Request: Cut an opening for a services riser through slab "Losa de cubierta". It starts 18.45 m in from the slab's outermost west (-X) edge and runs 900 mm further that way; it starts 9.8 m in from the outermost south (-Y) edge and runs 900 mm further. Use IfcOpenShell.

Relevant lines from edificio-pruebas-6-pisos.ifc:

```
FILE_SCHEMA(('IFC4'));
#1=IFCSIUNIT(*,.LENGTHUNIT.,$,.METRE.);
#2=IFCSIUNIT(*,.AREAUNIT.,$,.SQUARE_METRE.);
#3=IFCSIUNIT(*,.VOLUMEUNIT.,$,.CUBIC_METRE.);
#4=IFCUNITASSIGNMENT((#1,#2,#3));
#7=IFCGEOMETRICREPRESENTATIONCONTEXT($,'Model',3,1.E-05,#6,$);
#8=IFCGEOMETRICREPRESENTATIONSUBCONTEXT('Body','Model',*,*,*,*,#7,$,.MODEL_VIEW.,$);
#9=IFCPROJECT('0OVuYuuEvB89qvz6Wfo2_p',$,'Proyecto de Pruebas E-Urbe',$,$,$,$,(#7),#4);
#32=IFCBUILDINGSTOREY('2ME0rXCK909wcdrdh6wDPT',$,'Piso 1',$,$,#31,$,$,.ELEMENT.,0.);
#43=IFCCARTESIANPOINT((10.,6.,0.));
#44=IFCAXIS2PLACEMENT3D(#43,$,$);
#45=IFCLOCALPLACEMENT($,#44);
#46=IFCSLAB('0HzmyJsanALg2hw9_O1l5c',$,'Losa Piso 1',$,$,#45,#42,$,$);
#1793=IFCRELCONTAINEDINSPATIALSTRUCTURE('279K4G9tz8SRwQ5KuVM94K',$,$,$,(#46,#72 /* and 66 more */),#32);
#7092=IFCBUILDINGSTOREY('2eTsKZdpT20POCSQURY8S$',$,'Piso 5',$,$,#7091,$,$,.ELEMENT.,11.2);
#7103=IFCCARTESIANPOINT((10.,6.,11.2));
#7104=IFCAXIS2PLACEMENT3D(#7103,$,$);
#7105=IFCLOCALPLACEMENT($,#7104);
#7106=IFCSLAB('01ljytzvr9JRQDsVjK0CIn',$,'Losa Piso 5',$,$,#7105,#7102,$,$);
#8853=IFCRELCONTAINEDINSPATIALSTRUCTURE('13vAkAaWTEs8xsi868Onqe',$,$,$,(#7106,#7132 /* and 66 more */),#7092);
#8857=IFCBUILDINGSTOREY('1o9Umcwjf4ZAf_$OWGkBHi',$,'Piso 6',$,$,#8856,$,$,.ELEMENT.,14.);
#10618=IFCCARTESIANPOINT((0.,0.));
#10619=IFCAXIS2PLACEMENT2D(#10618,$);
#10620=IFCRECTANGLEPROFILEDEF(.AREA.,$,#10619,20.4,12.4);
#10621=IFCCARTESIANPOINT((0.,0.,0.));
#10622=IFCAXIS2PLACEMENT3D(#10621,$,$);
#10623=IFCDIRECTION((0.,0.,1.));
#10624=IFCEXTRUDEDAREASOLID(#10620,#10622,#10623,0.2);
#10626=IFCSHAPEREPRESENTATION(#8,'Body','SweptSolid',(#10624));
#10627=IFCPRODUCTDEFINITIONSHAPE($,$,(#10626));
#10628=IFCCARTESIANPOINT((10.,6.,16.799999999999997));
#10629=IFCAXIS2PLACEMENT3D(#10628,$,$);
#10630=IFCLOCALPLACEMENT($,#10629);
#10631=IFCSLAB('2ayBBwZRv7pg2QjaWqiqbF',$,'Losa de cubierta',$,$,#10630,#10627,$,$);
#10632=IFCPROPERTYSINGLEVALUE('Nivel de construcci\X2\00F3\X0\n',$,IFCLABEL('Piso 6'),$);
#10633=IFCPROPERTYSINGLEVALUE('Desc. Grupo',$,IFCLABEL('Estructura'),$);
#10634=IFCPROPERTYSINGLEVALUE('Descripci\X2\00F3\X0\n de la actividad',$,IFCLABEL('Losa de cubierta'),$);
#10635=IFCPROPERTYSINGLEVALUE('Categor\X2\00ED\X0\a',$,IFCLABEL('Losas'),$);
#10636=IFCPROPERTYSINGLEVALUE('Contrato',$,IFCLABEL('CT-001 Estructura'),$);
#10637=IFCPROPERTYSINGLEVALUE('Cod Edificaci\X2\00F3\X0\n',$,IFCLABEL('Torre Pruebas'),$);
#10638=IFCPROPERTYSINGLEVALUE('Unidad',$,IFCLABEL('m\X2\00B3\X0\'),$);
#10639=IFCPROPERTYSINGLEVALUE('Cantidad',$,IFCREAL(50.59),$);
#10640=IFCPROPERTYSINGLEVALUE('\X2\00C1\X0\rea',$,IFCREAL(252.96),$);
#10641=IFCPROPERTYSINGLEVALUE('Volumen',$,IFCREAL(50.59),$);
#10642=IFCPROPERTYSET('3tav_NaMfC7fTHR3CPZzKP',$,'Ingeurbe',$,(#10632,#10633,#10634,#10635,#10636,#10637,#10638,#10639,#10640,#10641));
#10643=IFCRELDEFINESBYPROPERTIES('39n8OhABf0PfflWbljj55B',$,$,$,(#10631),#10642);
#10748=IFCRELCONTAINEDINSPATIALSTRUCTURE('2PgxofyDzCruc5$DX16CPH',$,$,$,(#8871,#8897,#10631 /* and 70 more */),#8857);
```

```python
import numpy as np
import ifcopenshell
import ifcopenshell.api.feature
import ifcopenshell.api.geometry
import ifcopenshell.api.pset
import ifcopenshell.api.root
import ifcopenshell.geom
import ifcopenshell.util.element
import ifcopenshell.util.placement
import ifcopenshell.util.representation
import ifcopenshell.util.shape
import ifcopenshell.util.unit

model = ifcopenshell.open("edificio-pruebas-6-pisos.ifc")
unit_scale = ifcopenshell.util.unit.calculate_unit_scale(model)
area_scale = ifcopenshell.util.unit.calculate_unit_scale(model, "AREAUNIT")
volume_scale = ifcopenshell.util.unit.calculate_unit_scale(model, "VOLUMEUNIT")
settings = ifcopenshell.geom.settings()


def volume(element):
    """Net volume in cubic metres, openings subtracted."""
    shape = ifcopenshell.geom.create_shape(settings, element)
    return ifcopenshell.util.shape.get_volume(shape.geometry)


slab = model.by_guid("2ayBBwZRv7pg2QjaWqiqbF")
before = volume(slab)

# Extent in the slab's own axes, in metres. The edges named are its -X and -Y sides.
slab_shape = ifcopenshell.geom.create_shape(settings, slab)
vertices = ifcopenshell.util.shape.get_vertices(slab_shape.geometry)
x_min, y_min, bottom = vertices.min(axis=0)
top = vertices[:, 2].max()

opening = ifcopenshell.api.root.create_entity(model, ifc_class="IfcOpeningElement", name="Services riser opening", predefined_type="OPENING")
context = ifcopenshell.util.representation.get_context(model, "Model", "Body", "MODEL_VIEW")
width, depth = 0.9, 0.9
outline = [(0.0, 0.0), (width, 0.0), (width, depth), (0.0, depth), (0.0, 0.0)]
# Overshoot both faces by 50 mm so the cut is clean.
shape = ifcopenshell.api.geometry.add_slab_representation(
    model, context=context, depth=top - bottom + 0.1, polyline=outline
)
ifcopenshell.api.geometry.assign_representation(model, product=opening, representation=shape)

matrix = ifcopenshell.util.placement.get_local_placement(slab.ObjectPlacement)
matrix[:, 3] = matrix @ np.append(np.array([x_min + 18.45, y_min + 9.8, bottom - 0.05]) / unit_scale, 1.0)
ifcopenshell.api.geometry.edit_object_placement(model, product=opening, matrix=matrix, is_si=False)
ifcopenshell.api.feature.add_feature(model, feature=opening, element=slab)

after = volume(slab)

# Update the slab's stored quantities.
pset = model.by_id(ifcopenshell.util.element.get_pset(slab, "Ingeurbe", should_inherit=False)["id"])
ifcopenshell.api.pset.edit_pset(model, pset=pset, properties={
    "Área": model.create_entity("IfcReal", after / (top - bottom) / area_scale),
    "Volumen": model.create_entity("IfcReal", after / volume_scale),
})

print(f"slab volume {before:.3f} -> {after:.3f} m3")

model.write("edificio-pruebas-6-pisos_rev.ifc")
```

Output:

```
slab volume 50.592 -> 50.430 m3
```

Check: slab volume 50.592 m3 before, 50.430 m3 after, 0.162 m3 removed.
